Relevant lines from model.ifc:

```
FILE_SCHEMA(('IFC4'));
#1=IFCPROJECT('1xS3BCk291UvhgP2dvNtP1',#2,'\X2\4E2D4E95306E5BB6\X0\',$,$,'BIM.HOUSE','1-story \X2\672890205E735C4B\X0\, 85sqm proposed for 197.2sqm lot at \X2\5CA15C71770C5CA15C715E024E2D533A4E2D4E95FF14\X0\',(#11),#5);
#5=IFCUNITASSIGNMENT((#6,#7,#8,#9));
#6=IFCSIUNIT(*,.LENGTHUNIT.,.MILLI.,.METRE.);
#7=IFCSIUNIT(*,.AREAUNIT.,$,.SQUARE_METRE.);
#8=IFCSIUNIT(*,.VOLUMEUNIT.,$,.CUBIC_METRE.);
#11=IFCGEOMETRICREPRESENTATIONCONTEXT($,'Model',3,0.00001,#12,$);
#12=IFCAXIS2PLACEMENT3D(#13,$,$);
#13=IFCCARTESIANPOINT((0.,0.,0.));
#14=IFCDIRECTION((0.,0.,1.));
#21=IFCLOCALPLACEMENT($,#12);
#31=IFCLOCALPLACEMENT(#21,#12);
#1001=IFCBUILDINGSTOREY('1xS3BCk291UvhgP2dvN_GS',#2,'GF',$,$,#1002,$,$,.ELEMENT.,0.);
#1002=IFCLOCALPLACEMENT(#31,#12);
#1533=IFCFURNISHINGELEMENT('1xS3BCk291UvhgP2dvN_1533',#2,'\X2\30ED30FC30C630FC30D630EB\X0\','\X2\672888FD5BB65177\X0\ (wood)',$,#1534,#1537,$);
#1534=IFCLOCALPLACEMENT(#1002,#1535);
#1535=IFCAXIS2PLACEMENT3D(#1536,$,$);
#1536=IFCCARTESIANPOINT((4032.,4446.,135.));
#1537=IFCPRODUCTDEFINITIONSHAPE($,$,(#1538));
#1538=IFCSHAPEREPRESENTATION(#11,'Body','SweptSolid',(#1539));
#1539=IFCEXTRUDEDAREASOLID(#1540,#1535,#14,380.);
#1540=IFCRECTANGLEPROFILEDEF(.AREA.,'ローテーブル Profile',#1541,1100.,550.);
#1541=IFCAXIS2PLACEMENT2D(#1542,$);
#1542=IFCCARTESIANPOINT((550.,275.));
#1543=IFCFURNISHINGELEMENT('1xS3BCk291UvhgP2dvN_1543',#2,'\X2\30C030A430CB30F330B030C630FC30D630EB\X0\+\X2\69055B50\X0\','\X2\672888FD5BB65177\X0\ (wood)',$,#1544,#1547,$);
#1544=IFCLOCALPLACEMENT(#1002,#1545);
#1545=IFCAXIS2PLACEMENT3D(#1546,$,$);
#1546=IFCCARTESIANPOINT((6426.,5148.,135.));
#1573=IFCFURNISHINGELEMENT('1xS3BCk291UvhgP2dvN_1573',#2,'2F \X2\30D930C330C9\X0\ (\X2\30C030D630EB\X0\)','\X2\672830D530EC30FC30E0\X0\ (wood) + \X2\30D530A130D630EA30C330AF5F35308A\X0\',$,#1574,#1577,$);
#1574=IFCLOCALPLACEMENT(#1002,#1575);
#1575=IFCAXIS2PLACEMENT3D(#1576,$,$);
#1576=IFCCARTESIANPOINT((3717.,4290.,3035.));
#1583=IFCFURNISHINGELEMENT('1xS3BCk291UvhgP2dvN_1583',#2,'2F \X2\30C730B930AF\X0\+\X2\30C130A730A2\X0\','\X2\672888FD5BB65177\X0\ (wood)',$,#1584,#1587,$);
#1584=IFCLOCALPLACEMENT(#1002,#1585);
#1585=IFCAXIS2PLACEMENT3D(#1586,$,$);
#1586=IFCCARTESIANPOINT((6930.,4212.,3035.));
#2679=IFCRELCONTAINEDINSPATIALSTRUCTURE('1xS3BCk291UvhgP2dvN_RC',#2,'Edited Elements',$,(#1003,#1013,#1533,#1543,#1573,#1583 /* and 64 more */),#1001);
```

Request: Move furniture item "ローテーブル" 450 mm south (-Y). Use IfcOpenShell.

```python
import ifcopenshell
import ifcopenshell.api.geometry
import ifcopenshell.util.placement

model = ifcopenshell.open("model.ifc")

item = model.by_guid("1xS3BCk291UvhgP2dvN_1533")
matrix = ifcopenshell.util.placement.get_local_placement(item.ObjectPlacement)
matrix[1, 3] -= 450.0
ifcopenshell.api.geometry.edit_object_placement(model, product=item, matrix=matrix, is_si=False)

print(ifcopenshell.util.placement.get_local_placement(item.ObjectPlacement).round(3) + 0.0)

model.write("model_edited.ifc")
```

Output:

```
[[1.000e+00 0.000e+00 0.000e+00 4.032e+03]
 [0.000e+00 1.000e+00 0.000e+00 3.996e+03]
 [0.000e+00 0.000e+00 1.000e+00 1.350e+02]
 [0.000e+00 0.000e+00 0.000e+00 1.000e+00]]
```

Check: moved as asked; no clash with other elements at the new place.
